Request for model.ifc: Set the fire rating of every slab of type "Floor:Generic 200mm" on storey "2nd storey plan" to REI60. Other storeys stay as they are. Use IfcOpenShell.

First a look at what the model holds.

```python
import ifcopenshell
import ifcopenshell.util.element

model = ifcopenshell.open("model.ifc")
print(model.schema)
storey = next(s for s in model.by_type("IfcBuildingStorey") if s.Name == "2nd storey plan")
slabs = [e for e in ifcopenshell.util.element.get_decomposition(storey) if e.is_a("IfcSlab")]
seen = {}
for e in slabs:
    element_type = ifcopenshell.util.element.get_type(e)
    key = (element_type.Name if element_type != e and element_type else None, ifcopenshell.util.element.get_pset(e, "Pset_SlabCommon", "FireRating"))
    seen[key] = seen.get(key, 0) + 1
for (name, value), count in sorted(seen.items(), key=str):
    print(count, "x", name, "|", value)
```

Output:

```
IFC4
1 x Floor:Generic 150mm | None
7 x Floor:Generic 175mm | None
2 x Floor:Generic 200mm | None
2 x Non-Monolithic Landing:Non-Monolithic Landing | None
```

```python
import ifcopenshell
import ifcopenshell.api.pset
import ifcopenshell.util.element

model = ifcopenshell.open("model.ifc")

storey = next(s for s in model.by_type("IfcBuildingStorey") if s.Name == "2nd storey plan")
slabs = [e for e in ifcopenshell.util.element.get_decomposition(storey) if e.is_a("IfcSlab")]

count = 0
for e in slabs:
    element_type = ifcopenshell.util.element.get_type(e)
    if element_type in (None, e) or element_type.Name != "Floor:Generic 200mm":
        continue
    # add_pset returns the element's existing set when there is one.
    pset = ifcopenshell.api.pset.add_pset(model, product=e, name="Pset_SlabCommon")
    ifcopenshell.api.pset.edit_pset(model, pset=pset, properties={"FireRating": "REI60"})
    count += 1

print(count, "slabs updated")

model.write("model_rev.ifc")
```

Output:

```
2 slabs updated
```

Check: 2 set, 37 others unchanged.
